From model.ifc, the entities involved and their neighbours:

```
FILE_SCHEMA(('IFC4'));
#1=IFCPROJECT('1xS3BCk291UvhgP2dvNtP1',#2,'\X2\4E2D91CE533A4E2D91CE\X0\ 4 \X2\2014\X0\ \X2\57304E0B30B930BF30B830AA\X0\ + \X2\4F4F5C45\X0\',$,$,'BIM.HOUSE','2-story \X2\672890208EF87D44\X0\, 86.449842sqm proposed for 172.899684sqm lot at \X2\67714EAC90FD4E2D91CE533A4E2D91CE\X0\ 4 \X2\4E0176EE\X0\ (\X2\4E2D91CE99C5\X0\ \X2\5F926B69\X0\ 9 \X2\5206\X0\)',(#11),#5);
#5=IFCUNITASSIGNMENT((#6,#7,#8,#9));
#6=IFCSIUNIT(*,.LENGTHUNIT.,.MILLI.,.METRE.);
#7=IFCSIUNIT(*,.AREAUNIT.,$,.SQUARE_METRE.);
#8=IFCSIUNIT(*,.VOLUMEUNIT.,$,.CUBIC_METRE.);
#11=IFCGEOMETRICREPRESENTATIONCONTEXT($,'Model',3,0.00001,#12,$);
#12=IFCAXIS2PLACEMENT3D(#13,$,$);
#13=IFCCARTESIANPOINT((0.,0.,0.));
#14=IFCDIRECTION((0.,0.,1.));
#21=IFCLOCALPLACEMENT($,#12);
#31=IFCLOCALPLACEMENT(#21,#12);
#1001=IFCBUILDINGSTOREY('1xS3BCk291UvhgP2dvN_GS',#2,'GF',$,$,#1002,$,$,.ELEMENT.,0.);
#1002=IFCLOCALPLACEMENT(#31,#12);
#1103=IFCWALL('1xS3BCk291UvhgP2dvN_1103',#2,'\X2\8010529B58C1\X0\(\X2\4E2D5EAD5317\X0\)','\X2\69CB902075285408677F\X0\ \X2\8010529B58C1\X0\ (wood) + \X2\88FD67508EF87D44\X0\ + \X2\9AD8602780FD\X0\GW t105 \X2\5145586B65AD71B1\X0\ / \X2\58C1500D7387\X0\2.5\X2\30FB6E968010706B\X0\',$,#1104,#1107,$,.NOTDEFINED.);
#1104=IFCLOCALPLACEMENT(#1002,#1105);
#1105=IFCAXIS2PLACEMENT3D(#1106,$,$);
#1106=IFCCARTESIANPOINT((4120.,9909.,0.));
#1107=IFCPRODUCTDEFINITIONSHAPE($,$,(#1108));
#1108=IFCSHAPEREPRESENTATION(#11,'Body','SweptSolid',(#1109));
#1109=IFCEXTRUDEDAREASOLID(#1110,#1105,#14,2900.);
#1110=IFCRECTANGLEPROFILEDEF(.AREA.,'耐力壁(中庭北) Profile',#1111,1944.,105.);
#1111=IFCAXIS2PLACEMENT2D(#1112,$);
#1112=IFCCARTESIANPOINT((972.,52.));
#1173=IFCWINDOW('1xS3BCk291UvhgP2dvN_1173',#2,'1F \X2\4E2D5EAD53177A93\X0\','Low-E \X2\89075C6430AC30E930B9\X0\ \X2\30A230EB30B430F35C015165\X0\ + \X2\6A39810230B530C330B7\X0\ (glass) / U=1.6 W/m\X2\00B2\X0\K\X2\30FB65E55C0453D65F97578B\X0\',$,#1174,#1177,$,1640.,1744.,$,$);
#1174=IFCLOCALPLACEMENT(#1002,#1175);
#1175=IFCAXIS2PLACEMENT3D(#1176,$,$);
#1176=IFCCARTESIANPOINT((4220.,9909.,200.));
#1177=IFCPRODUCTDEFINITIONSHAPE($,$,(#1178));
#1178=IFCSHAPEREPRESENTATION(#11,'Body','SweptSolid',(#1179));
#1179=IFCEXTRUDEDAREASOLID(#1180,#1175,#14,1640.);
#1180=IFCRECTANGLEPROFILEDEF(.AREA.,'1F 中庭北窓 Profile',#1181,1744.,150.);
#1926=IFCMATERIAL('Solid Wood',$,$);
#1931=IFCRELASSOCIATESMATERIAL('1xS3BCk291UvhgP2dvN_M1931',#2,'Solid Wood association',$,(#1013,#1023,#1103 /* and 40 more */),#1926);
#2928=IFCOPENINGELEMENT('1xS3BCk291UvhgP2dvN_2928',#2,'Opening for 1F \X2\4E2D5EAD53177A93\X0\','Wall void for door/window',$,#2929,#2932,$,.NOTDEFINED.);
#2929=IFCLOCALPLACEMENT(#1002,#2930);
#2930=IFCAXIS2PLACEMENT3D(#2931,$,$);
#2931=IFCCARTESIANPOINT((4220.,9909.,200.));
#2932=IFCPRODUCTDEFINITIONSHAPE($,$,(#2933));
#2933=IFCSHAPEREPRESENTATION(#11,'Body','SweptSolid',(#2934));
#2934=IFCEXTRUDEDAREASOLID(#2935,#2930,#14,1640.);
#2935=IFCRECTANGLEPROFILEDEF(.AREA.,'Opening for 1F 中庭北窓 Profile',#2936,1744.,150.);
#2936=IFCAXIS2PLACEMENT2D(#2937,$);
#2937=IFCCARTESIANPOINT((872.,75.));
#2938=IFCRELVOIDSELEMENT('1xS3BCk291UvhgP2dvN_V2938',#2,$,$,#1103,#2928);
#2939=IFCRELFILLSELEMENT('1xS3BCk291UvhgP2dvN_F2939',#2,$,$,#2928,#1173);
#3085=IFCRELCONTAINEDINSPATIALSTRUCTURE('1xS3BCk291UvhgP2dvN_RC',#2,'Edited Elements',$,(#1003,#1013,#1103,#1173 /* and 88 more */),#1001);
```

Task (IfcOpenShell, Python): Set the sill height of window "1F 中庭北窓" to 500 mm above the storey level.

```python
import numpy as np
import ifcopenshell
import ifcopenshell.api.geometry
import ifcopenshell.geom
import ifcopenshell.util.element
import ifcopenshell.util.placement
import ifcopenshell.util.shape
import ifcopenshell.util.unit

model = ifcopenshell.open("model.ifc")
unit_scale = ifcopenshell.util.unit.calculate_unit_scale(model)

window = model.by_guid("1xS3BCk291UvhgP2dvN_1173")
opening = window.FillsVoids[0].RelatingOpeningElement
storey = ifcopenshell.util.element.get_container(window, ifc_class="IfcBuildingStorey")
level = ifcopenshell.util.placement.get_local_placement(storey.ObjectPlacement)[2, 3]

# The opening's origin need not be at the sill, so measure its lowest point.
shape = ifcopenshell.geom.create_shape(ifcopenshell.geom.settings(), opening)
bottom = ifcopenshell.util.shape.get_shape_bottom_elevation(shape, shape.geometry) / unit_scale
dz = level + 0.5 / unit_scale - bottom

shift = np.array([0.0, 0.0, dz])
# The window is not placed relative to its opening, so move both.
for product in (opening, window):
    matrix = ifcopenshell.util.placement.get_local_placement(product.ObjectPlacement)
    matrix[:3, 3] += shift
    ifcopenshell.api.geometry.edit_object_placement(model, product=product, matrix=matrix, is_si=False)

print(f"moved by {dz * unit_scale:+.3f} m")

model.write("model_v2.ifc")
```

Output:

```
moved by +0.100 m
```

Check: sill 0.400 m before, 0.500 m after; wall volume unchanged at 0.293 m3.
